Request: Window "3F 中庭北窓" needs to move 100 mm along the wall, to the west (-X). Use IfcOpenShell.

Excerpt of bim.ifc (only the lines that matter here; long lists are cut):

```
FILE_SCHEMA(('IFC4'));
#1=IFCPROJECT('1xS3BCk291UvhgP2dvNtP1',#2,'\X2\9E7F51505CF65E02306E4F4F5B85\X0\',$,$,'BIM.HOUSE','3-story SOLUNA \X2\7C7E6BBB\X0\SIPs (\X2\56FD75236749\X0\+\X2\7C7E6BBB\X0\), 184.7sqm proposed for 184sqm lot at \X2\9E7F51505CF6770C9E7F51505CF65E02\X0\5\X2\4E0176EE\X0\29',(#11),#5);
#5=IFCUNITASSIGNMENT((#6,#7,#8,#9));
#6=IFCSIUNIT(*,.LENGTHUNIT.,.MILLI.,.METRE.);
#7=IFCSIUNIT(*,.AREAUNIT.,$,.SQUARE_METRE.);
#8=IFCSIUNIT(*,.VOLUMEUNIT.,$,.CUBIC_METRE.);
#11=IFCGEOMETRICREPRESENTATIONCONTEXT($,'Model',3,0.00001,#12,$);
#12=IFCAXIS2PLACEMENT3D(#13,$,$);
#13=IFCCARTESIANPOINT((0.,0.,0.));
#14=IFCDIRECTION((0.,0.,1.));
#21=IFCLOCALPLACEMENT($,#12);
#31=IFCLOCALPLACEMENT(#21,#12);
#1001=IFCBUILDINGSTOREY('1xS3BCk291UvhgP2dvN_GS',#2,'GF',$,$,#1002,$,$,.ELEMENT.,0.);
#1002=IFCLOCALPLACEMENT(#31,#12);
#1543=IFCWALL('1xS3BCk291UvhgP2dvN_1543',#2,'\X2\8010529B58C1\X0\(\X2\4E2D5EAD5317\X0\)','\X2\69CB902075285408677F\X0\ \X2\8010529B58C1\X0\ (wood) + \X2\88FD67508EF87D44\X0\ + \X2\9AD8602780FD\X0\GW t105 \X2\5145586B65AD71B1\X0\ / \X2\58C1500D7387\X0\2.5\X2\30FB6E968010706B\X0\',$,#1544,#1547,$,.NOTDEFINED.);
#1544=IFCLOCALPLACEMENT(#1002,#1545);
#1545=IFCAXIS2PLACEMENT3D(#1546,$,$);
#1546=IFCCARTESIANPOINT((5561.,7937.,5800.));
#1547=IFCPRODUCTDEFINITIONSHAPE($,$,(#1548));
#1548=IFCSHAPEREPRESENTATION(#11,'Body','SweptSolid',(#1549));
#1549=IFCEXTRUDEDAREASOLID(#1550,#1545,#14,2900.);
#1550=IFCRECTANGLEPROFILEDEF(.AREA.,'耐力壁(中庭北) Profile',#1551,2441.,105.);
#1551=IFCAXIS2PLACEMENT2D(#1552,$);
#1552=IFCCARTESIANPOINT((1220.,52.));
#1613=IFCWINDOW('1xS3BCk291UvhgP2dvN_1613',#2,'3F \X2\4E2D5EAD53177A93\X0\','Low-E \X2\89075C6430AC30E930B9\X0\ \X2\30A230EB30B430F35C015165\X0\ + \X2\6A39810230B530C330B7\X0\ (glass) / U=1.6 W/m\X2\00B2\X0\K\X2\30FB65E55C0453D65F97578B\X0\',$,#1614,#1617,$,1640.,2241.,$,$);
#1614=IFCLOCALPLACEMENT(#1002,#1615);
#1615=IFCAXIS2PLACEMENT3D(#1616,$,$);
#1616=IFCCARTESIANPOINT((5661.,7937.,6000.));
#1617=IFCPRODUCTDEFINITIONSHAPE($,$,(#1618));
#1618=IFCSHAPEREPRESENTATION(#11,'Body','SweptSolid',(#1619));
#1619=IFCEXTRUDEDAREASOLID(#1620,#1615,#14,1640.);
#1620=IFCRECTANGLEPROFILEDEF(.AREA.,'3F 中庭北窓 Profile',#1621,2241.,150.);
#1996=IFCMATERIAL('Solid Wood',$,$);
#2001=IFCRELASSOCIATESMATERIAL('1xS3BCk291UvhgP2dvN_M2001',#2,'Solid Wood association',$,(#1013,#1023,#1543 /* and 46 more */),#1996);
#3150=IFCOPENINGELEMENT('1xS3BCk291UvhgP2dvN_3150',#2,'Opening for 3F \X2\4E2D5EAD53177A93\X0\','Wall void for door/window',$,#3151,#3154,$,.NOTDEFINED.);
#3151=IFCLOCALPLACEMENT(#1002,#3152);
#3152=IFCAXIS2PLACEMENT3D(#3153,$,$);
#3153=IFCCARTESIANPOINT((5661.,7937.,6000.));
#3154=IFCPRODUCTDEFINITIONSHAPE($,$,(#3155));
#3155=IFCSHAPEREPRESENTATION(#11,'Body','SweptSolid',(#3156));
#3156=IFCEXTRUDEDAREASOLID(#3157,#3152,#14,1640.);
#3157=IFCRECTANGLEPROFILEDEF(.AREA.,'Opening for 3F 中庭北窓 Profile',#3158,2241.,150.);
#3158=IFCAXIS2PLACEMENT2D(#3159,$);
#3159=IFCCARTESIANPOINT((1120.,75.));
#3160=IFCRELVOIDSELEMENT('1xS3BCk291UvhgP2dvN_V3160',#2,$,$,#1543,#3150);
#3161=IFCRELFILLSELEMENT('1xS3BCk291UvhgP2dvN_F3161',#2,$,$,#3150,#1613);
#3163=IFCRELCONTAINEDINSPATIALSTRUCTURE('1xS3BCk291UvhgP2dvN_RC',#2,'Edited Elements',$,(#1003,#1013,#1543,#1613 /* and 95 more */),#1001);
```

```python
import ifcopenshell
import ifcopenshell.api.geometry
import ifcopenshell.util.placement
import ifcopenshell.util.unit

model = ifcopenshell.open("bim.ifc")
unit_scale = ifcopenshell.util.unit.calculate_unit_scale(model)

window = model.by_guid("1xS3BCk291UvhgP2dvN_1613")
opening = window.FillsVoids[0].RelatingOpeningElement
wall = opening.VoidsElements[0].RelatingBuildingElement

wall_matrix = ifcopenshell.util.placement.get_local_placement(wall.ObjectPlacement)
shift = wall_matrix[:3, 0] * -0.1 / unit_scale
before = ifcopenshell.util.placement.get_local_placement(window.ObjectPlacement)[:3, 3].copy()

# The window is not placed relative to its opening, so move both.
for product in (opening, window):
    matrix = ifcopenshell.util.placement.get_local_placement(product.ObjectPlacement)
    matrix[:3, 3] += shift
    ifcopenshell.api.geometry.edit_object_placement(model, product=product, matrix=matrix, is_si=False)

after = ifcopenshell.util.placement.get_local_placement(window.ObjectPlacement)[:3, 3]
print("window moved by", (after - before).round(3) + 0.0)

model.write("bim_rev.ifc")
```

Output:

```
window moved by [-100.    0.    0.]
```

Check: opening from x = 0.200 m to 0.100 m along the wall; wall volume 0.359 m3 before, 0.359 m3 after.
